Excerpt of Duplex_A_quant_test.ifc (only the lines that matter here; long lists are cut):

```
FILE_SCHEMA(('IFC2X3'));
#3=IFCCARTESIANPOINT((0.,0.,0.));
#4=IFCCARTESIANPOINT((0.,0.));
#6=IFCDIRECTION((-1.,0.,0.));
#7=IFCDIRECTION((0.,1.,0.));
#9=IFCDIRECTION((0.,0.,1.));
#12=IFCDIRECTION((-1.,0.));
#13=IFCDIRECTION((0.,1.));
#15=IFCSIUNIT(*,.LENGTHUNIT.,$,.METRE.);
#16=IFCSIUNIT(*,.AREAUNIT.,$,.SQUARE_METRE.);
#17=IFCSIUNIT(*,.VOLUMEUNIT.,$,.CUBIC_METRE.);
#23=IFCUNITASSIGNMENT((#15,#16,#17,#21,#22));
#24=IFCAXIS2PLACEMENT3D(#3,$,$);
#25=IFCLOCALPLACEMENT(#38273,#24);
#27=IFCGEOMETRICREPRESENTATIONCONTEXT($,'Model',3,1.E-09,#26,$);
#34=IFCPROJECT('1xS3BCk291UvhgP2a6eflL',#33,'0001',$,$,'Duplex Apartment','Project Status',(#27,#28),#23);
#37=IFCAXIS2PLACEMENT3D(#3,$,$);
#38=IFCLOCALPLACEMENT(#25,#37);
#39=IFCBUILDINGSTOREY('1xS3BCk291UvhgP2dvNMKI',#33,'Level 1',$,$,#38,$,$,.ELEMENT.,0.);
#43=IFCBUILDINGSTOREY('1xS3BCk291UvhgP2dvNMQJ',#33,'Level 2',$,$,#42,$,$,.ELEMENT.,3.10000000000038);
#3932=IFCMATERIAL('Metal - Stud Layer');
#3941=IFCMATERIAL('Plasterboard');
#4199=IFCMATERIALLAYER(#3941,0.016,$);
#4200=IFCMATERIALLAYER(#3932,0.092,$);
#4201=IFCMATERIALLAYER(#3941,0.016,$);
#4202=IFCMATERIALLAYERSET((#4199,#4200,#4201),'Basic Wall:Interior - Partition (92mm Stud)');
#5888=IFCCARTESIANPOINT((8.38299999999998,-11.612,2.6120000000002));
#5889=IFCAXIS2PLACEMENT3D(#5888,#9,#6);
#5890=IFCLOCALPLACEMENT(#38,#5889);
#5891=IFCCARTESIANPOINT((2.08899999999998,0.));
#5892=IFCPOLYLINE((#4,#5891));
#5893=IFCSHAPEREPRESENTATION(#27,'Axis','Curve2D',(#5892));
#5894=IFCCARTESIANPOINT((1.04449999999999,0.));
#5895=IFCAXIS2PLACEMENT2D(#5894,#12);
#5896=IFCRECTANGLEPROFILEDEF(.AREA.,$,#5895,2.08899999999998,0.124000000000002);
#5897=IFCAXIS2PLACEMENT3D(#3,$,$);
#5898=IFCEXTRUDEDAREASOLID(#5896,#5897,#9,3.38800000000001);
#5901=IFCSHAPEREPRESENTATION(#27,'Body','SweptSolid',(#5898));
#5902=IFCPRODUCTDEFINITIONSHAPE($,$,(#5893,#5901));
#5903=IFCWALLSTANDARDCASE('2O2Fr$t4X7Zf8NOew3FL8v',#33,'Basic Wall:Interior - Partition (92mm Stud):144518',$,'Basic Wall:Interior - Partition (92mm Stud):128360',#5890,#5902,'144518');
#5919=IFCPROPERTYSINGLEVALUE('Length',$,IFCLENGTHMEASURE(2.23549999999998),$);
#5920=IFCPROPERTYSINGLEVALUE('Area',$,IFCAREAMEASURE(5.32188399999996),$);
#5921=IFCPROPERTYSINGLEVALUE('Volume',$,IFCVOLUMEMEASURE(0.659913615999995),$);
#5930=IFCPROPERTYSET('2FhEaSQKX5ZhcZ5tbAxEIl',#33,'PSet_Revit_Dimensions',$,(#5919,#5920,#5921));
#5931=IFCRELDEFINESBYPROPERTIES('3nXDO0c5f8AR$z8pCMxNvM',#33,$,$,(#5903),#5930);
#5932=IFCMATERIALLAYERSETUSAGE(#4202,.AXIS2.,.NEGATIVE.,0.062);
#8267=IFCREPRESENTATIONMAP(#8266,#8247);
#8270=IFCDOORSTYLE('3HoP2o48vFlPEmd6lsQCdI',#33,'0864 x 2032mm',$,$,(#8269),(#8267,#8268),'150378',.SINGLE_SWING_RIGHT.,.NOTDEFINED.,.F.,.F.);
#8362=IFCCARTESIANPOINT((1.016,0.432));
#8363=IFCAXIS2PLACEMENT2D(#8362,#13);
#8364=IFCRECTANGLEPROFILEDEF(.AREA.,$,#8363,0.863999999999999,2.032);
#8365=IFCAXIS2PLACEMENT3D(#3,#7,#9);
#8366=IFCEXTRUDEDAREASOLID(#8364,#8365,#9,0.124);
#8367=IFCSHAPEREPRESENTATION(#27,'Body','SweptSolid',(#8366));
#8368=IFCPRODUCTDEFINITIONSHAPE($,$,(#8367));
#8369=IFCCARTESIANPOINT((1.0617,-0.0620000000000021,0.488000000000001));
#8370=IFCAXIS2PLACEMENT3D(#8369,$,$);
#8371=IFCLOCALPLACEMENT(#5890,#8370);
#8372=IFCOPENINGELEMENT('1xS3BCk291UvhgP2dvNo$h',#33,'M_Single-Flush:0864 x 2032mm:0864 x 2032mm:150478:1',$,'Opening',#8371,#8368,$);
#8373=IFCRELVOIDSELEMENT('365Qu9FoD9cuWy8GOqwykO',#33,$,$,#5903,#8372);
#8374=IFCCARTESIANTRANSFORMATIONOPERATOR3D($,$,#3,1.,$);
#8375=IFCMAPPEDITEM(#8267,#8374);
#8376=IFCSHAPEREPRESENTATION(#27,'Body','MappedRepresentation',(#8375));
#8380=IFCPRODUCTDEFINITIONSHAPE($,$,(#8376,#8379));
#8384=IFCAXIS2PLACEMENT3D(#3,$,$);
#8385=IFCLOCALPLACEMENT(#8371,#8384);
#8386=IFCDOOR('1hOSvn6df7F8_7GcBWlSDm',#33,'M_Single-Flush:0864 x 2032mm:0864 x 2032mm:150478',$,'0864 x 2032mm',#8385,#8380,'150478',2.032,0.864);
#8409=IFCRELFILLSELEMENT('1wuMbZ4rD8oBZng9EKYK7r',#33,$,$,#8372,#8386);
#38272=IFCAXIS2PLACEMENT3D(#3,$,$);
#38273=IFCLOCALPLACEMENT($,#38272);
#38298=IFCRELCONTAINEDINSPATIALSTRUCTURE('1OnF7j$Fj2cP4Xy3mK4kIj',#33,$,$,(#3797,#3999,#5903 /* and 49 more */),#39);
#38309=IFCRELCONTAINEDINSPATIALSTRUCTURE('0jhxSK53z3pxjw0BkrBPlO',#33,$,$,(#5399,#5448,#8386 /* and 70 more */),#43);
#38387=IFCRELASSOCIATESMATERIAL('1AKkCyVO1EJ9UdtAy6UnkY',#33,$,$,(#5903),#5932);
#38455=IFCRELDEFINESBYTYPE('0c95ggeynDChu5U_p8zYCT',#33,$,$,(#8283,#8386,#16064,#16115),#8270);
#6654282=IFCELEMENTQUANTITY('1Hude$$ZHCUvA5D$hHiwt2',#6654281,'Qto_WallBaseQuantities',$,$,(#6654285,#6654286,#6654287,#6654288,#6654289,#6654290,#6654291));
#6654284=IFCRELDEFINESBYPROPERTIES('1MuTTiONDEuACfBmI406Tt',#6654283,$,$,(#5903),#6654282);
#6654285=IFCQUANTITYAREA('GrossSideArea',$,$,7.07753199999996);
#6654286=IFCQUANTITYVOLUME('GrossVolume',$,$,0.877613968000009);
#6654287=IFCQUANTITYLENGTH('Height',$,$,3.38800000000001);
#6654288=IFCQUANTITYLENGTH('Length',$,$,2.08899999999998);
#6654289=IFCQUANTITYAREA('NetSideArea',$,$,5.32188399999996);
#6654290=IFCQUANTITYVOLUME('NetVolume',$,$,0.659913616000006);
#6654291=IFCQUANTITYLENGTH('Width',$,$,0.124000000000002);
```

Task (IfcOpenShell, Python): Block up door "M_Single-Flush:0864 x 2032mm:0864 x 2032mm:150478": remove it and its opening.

```python
import ifcopenshell
import ifcopenshell.api.feature
import ifcopenshell.api.pset
import ifcopenshell.api.root
import ifcopenshell.geom
import ifcopenshell.util.element
import ifcopenshell.util.shape
import ifcopenshell.util.unit

model = ifcopenshell.open("Duplex_A_quant_test.ifc")
area_scale = ifcopenshell.util.unit.calculate_unit_scale(model, "AREAUNIT")
volume_scale = ifcopenshell.util.unit.calculate_unit_scale(model, "VOLUMEUNIT")
settings = ifcopenshell.geom.settings()


def volume(element):
    """Net volume in cubic metres, openings subtracted."""
    shape = ifcopenshell.geom.create_shape(settings, element)
    return ifcopenshell.util.shape.get_volume(shape.geometry)


door = model.by_guid("1hOSvn6df7F8_7GcBWlSDm")
opening = door.FillsVoids[0].RelatingOpeningElement
wall = opening.VoidsElements[0].RelatingBuildingElement
before = volume(wall)

ifcopenshell.api.root.remove_product(model, product=door)
ifcopenshell.api.feature.remove_feature(model, feature=opening)

after = volume(wall)
thickness = 0.124  # wall thickness in metres

# Update the wall's stored quantities.
pset = model.by_id(ifcopenshell.util.element.get_pset(wall, "PSet_Revit_Dimensions", should_inherit=False)["id"])
ifcopenshell.api.pset.edit_pset(model, pset=pset, properties={
    "Area": model.create_entity("IfcAreaMeasure", after / thickness / area_scale),
    "Volume": model.create_entity("IfcVolumeMeasure", after / volume_scale),
})
qto = model.by_id(ifcopenshell.util.element.get_pset(wall, "Qto_WallBaseQuantities", should_inherit=False)["id"])
ifcopenshell.api.pset.edit_qto(model, qto=qto, properties={
    "NetSideArea": after / thickness / area_scale,
    "NetVolume": after / volume_scale,
})

print(f"wall volume {before:.3f} -> {after:.3f} m3")

model.write("Duplex_A_quant_test_rev.ifc")
```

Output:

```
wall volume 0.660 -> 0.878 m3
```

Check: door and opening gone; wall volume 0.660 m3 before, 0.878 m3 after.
